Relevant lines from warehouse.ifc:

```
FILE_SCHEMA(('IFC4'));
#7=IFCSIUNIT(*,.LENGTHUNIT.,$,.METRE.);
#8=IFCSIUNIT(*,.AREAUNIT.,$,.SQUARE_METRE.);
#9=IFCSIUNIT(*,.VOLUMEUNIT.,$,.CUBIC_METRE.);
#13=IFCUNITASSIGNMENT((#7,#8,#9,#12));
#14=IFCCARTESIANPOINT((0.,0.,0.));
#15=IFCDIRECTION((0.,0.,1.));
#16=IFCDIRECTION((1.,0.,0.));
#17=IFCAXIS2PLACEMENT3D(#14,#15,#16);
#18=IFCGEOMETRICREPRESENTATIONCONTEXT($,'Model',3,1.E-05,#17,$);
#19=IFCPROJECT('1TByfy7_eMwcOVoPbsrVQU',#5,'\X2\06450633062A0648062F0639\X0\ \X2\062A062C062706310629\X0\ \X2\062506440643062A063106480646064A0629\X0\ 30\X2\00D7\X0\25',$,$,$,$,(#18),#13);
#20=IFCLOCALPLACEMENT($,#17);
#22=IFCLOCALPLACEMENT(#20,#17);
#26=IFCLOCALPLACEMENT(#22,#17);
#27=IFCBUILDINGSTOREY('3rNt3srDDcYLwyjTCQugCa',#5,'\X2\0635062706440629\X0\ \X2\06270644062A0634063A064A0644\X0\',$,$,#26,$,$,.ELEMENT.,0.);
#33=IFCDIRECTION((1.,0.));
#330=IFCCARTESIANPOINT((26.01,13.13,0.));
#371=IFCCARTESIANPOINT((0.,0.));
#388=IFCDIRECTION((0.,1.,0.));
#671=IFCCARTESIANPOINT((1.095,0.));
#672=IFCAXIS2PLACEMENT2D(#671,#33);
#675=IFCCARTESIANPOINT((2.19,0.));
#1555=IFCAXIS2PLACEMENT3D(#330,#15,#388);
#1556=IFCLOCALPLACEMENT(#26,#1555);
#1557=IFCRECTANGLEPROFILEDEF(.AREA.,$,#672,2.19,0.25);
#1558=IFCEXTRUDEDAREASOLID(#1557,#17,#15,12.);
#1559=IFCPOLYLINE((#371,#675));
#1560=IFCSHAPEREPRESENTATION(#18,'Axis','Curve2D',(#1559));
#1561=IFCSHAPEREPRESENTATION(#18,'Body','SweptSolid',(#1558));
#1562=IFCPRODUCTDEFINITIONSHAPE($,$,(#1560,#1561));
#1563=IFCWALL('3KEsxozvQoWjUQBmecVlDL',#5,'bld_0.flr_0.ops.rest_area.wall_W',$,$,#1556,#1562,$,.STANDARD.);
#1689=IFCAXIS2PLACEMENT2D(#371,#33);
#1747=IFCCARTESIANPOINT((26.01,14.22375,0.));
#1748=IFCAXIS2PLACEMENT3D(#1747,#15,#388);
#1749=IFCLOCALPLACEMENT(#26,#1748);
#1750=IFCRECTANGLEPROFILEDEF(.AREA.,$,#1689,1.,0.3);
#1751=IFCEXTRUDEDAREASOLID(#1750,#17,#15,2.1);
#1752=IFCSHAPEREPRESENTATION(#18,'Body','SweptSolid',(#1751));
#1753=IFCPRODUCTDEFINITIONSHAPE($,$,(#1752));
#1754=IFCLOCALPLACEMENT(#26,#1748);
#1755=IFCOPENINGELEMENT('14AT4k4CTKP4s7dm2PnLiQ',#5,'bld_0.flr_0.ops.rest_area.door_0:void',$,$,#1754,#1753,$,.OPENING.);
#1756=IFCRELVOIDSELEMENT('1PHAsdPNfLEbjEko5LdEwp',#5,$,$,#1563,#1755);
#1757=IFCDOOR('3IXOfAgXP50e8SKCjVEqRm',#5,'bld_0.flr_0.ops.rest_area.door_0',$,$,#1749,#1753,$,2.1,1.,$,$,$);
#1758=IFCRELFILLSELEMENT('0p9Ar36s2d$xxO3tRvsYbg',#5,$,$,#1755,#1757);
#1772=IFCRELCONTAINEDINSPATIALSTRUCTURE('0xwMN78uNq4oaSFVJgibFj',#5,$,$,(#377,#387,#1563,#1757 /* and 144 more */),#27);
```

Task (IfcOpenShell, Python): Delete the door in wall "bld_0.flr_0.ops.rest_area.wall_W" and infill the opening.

```python
import ifcopenshell
import ifcopenshell.api.feature
import ifcopenshell.api.root
import ifcopenshell.geom
import ifcopenshell.util.shape

model = ifcopenshell.open("warehouse.ifc")
settings = ifcopenshell.geom.settings()


def volume(element):
    """Net volume in cubic metres, openings subtracted."""
    shape = ifcopenshell.geom.create_shape(settings, element)
    return ifcopenshell.util.shape.get_volume(shape.geometry)


door = model.by_guid("3IXOfAgXP50e8SKCjVEqRm")
opening = door.FillsVoids[0].RelatingOpeningElement
wall = opening.VoidsElements[0].RelatingBuildingElement
before = volume(wall)

ifcopenshell.api.root.remove_product(model, product=door)
ifcopenshell.api.feature.remove_feature(model, feature=opening)

after = volume(wall)

print(f"wall volume {before:.3f} -> {after:.3f} m3")

model.write("warehouse_rev.ifc")
```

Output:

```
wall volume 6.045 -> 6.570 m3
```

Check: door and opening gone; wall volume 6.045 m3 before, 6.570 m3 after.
